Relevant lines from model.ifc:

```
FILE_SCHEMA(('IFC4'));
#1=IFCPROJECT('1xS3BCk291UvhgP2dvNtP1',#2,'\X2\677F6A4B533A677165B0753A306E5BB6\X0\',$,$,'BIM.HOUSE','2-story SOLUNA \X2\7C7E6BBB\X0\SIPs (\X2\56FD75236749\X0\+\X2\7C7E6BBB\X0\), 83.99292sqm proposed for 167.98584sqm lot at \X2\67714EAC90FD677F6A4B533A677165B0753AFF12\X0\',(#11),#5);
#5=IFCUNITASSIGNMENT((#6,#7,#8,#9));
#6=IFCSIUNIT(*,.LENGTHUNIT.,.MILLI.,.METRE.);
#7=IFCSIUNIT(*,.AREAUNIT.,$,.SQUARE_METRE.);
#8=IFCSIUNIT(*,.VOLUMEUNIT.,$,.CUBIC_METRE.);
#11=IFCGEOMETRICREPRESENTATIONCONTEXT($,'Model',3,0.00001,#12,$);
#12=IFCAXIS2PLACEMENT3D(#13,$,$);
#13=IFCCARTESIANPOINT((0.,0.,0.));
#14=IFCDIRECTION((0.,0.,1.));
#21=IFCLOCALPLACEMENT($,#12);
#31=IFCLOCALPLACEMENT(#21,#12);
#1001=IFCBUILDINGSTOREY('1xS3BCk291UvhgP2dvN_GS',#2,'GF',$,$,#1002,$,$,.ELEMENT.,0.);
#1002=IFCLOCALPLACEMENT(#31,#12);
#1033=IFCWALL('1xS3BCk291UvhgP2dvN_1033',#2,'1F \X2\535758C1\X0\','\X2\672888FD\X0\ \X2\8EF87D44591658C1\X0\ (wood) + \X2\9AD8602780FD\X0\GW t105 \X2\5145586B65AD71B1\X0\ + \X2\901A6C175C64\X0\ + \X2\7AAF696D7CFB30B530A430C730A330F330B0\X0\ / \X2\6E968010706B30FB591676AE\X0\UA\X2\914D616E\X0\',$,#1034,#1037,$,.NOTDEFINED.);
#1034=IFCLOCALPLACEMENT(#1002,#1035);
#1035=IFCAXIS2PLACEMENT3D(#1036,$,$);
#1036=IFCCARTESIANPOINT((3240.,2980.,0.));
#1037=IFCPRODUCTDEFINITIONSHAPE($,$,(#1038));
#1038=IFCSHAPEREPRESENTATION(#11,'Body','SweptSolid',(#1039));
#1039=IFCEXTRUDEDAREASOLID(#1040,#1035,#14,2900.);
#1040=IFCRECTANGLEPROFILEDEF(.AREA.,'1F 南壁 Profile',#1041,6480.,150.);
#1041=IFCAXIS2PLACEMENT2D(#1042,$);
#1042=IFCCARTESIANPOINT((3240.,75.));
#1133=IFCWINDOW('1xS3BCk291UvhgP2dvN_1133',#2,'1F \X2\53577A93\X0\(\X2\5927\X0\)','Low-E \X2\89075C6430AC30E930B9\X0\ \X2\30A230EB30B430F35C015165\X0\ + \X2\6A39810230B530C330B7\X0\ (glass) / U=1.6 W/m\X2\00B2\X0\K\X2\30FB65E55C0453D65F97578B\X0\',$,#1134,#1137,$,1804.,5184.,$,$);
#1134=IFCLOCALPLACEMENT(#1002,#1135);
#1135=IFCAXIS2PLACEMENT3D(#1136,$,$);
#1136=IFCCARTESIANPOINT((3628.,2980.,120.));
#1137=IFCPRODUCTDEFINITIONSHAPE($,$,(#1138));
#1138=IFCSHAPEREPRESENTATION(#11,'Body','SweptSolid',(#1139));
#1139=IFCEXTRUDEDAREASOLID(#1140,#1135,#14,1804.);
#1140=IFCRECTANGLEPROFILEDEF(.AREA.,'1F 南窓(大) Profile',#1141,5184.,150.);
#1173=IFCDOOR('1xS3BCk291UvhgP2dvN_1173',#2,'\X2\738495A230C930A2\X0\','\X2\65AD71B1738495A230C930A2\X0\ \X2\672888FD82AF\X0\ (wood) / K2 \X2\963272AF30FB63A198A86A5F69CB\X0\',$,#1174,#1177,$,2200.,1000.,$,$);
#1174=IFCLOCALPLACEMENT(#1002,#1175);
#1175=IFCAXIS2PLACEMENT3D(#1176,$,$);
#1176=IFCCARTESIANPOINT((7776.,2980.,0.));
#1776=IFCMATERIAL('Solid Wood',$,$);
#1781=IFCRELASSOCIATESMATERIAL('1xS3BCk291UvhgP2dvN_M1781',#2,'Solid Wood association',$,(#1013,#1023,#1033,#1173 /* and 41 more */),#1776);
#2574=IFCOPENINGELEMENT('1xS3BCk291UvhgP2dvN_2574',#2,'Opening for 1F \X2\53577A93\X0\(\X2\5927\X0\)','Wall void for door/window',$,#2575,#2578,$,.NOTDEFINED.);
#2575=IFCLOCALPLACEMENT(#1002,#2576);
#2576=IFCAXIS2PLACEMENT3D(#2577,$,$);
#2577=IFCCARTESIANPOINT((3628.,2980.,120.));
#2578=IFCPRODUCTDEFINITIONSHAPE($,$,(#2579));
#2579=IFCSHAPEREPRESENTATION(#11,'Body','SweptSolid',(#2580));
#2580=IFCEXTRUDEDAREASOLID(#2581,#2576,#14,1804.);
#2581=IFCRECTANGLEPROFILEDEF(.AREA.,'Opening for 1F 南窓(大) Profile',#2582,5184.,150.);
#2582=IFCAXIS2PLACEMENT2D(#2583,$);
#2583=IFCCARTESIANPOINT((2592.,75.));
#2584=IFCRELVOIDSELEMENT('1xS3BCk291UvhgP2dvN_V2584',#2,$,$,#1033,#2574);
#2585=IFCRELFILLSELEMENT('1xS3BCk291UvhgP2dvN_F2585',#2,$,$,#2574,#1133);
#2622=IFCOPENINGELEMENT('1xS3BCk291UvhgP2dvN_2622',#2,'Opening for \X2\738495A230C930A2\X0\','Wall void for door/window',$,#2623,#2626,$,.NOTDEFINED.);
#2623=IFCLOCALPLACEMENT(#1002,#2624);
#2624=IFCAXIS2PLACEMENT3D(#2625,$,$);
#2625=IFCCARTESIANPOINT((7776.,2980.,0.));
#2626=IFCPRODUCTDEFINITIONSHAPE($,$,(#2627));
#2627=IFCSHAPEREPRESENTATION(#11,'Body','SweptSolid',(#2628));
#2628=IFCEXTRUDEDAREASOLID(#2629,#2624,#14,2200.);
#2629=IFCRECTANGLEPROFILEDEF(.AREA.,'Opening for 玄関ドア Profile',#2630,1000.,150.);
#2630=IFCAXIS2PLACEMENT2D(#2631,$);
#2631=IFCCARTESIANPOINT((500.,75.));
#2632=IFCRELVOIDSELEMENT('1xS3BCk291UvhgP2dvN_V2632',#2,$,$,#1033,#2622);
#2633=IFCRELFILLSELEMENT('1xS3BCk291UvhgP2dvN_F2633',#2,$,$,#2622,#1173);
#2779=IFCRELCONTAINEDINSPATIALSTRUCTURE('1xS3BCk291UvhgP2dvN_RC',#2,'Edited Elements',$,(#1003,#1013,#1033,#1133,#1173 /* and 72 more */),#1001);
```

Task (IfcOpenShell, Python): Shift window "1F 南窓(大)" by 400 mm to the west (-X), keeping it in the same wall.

```python
import ifcopenshell
import ifcopenshell.api.geometry
import ifcopenshell.util.placement

model = ifcopenshell.open("model.ifc")

window = model.by_guid("1xS3BCk291UvhgP2dvN_1133")
opening = window.FillsVoids[0].RelatingOpeningElement
wall = opening.VoidsElements[0].RelatingBuildingElement

wall_matrix = ifcopenshell.util.placement.get_local_placement(wall.ObjectPlacement)
shift = wall_matrix[:3, 0] * -400.0
before = ifcopenshell.util.placement.get_local_placement(window.ObjectPlacement)[:3, 3].copy()

# The window is not placed relative to its opening, so move both.
for product in (opening, window):
    matrix = ifcopenshell.util.placement.get_local_placement(product.ObjectPlacement)
    matrix[:3, 3] += shift
    ifcopenshell.api.geometry.edit_object_placement(model, product=product, matrix=matrix, is_si=False)

after = ifcopenshell.util.placement.get_local_placement(window.ObjectPlacement)[:3, 3]
print("window moved by", (after - before).round(3) + 0.0)

model.write("model-out.ifc")
```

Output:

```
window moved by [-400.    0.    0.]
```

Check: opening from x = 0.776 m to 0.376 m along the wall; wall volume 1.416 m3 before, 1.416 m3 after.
